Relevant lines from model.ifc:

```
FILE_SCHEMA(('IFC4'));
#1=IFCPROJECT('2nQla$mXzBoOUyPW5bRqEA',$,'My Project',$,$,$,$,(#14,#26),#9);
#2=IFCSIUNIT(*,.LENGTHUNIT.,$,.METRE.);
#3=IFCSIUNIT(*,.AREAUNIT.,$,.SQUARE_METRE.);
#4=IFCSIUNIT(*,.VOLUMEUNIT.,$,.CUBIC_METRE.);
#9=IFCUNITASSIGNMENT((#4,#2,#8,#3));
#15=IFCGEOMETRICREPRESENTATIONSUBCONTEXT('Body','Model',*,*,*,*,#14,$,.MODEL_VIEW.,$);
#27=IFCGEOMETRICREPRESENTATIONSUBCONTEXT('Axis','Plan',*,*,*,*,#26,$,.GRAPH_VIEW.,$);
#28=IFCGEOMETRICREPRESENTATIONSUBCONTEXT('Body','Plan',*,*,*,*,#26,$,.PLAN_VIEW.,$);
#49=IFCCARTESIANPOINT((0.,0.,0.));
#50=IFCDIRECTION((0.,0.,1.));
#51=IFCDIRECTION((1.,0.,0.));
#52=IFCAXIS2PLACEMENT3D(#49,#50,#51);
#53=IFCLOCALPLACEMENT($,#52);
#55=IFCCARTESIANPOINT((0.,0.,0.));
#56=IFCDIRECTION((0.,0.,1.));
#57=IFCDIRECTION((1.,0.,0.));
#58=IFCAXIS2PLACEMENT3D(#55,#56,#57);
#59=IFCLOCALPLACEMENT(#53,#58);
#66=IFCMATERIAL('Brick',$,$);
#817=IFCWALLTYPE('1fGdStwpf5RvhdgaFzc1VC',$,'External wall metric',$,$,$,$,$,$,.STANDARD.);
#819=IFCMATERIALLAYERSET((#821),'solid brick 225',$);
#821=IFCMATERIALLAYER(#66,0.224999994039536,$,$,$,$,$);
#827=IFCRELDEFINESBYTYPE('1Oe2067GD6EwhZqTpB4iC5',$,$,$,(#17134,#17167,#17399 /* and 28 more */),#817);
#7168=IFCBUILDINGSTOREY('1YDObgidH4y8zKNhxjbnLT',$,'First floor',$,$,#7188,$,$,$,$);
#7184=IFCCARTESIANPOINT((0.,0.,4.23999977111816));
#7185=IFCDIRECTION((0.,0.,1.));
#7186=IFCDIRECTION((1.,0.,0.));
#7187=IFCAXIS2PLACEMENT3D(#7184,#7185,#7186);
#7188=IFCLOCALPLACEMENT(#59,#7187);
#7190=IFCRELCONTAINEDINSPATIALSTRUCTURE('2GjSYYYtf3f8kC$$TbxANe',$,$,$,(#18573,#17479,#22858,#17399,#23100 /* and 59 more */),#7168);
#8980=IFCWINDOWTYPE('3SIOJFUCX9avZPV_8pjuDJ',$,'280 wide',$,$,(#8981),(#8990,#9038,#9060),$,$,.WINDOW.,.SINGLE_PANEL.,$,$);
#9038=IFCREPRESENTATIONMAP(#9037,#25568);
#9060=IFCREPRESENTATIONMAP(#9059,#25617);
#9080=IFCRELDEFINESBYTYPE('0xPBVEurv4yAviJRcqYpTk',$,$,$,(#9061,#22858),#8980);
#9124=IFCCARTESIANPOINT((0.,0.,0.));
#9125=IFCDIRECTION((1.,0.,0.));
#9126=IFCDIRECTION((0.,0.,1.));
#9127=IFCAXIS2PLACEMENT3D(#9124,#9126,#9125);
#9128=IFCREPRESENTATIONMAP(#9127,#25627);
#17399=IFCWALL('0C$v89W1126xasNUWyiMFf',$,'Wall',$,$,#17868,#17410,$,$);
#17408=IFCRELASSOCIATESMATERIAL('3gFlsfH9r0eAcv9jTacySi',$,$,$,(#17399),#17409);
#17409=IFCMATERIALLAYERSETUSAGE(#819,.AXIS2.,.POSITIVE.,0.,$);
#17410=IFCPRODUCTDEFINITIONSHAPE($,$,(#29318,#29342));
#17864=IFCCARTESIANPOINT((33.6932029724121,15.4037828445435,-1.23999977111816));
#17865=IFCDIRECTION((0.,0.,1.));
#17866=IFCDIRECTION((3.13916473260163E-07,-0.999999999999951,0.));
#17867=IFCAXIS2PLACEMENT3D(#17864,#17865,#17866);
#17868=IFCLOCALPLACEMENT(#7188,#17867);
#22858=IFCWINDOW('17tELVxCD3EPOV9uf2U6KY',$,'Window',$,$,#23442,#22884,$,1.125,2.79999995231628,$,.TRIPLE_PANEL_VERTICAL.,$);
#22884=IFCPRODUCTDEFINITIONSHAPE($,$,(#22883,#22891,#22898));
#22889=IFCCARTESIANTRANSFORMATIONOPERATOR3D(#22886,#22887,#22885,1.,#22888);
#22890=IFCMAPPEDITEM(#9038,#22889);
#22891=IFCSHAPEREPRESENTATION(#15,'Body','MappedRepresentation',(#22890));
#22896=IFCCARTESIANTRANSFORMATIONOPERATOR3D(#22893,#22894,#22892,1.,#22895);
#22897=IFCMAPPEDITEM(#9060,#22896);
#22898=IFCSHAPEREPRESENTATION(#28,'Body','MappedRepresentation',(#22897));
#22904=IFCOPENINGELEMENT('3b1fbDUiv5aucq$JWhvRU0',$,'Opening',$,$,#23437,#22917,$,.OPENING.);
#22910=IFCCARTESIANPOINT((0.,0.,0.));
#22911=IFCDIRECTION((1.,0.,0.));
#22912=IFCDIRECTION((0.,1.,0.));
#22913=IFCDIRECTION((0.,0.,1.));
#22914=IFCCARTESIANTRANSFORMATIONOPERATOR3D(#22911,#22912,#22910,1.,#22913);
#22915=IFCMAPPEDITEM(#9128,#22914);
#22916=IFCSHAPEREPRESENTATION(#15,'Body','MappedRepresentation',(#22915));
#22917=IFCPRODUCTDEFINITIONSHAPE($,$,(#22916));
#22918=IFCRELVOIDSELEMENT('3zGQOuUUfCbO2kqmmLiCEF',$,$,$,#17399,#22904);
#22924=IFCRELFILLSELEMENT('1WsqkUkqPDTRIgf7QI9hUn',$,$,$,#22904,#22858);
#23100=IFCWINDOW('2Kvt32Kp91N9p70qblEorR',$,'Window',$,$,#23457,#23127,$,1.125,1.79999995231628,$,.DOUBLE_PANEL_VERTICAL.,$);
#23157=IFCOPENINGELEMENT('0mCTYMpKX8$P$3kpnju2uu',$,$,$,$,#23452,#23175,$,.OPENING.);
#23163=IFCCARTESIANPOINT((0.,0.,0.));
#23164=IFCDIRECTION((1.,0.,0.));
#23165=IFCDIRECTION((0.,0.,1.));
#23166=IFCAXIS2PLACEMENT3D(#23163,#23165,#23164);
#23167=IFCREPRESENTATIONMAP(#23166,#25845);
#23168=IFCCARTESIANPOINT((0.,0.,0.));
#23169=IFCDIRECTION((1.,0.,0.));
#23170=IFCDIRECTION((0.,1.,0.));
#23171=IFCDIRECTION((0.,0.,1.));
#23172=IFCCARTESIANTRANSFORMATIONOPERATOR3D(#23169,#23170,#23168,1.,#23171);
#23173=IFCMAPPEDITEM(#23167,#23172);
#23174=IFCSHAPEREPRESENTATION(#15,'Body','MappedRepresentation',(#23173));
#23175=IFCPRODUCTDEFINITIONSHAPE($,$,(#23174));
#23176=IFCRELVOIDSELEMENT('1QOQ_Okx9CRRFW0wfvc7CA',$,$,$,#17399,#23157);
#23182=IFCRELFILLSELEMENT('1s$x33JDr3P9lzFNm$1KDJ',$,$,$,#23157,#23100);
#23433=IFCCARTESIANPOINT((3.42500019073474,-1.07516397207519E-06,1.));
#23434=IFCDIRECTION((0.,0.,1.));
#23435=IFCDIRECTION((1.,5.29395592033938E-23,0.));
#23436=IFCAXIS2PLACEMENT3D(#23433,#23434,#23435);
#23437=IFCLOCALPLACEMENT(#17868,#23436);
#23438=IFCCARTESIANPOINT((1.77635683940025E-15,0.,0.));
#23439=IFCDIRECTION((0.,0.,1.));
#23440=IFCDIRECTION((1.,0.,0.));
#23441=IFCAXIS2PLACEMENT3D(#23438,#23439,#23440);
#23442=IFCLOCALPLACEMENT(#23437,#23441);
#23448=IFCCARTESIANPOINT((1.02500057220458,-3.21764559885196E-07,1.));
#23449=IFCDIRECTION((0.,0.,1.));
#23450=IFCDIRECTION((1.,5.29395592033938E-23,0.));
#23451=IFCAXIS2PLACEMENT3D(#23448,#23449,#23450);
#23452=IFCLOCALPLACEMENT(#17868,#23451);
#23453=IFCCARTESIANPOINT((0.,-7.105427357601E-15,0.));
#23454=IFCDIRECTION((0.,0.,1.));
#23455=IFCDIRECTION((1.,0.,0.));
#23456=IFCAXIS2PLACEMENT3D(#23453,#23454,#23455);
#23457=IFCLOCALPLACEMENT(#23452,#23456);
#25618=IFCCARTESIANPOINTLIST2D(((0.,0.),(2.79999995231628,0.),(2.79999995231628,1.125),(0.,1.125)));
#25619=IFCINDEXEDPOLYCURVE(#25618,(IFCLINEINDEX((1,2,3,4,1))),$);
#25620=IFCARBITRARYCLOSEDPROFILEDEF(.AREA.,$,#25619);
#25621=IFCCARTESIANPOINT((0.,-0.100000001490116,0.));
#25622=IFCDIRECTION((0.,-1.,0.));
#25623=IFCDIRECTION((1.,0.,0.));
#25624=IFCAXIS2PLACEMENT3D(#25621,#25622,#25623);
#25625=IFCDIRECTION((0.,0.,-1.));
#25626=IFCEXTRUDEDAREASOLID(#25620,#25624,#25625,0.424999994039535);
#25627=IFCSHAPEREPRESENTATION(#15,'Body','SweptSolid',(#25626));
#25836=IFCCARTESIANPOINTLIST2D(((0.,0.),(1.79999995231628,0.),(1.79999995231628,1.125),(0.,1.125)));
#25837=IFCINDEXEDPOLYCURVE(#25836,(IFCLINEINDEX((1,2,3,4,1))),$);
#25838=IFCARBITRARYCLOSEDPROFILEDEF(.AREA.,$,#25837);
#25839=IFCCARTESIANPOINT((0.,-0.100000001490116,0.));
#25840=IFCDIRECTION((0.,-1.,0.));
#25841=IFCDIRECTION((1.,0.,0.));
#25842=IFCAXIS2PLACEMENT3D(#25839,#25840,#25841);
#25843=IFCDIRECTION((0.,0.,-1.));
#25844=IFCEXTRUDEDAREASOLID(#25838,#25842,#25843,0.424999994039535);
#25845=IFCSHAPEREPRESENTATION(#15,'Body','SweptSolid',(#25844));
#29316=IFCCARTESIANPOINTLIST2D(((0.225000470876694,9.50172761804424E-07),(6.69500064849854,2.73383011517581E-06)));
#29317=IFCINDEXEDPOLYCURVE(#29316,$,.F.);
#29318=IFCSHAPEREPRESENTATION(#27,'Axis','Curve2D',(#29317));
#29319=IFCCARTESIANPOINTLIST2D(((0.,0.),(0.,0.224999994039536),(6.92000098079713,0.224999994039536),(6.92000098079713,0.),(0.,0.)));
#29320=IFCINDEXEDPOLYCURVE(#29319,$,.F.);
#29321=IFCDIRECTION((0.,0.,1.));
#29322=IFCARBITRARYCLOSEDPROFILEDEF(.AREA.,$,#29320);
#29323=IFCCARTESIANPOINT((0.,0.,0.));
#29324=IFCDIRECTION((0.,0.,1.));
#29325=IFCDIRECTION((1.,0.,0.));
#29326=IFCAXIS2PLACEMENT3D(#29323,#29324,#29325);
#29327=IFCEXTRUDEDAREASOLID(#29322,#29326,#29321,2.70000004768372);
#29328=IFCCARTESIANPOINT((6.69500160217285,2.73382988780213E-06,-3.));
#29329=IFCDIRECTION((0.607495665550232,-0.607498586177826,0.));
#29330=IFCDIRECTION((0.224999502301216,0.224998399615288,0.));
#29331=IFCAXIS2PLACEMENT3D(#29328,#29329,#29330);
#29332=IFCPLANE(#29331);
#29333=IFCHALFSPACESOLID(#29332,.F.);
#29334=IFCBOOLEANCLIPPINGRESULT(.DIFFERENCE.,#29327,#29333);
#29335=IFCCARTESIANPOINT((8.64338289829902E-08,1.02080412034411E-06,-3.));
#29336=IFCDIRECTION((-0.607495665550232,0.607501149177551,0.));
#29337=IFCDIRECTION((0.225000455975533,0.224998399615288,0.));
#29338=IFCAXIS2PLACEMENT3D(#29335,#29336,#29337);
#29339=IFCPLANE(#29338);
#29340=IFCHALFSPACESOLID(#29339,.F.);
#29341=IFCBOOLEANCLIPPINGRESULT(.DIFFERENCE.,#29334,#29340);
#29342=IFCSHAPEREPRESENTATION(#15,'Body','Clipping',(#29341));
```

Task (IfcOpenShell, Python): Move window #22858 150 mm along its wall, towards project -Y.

```python
import ifcopenshell
import ifcopenshell.api.geometry
import ifcopenshell.util.placement

model = ifcopenshell.open("model.ifc")

window = model.by_guid("17tELVxCD3EPOV9uf2U6KY")
opening = window.FillsVoids[0].RelatingOpeningElement
wall = opening.VoidsElements[0].RelatingBuildingElement

wall_matrix = ifcopenshell.util.placement.get_local_placement(wall.ObjectPlacement)
shift = wall_matrix[:3, 0] * 0.15
before = ifcopenshell.util.placement.get_local_placement(window.ObjectPlacement)[:3, 3].copy()

# The window is placed relative to its opening, so it follows when the opening moves.
matrix = ifcopenshell.util.placement.get_local_placement(opening.ObjectPlacement)
matrix[:3, 3] += shift
ifcopenshell.api.geometry.edit_object_placement(
    model, product=opening, matrix=matrix, is_si=False, should_transform_children=True
)

after = ifcopenshell.util.placement.get_local_placement(window.ObjectPlacement)[:3, 3]
print("window moved by", (after - before).round(3) + 0.0)

model.write("model_updated.ifc")
```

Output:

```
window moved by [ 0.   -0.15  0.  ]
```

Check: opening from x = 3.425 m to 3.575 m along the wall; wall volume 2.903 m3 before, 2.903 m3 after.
